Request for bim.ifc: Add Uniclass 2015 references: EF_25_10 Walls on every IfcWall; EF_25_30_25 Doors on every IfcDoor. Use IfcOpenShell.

First a look at what the model holds.

```python
import ifcopenshell

model = ifcopenshell.open("bim.ifc")
print(model.schema)
print("classifications:", [c.Name for c in model.by_type("IfcClassification")])
for ifc_class in ("IfcDoor", "IfcRoof", "IfcStair", "IfcWall", "IfcWindow"):
    print(ifc_class, len(model.by_type(ifc_class)))
```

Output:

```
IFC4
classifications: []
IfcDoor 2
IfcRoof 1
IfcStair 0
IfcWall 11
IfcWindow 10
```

```python
import ifcopenshell
import ifcopenshell.api.classification

model = ifcopenshell.open("bim.ifc")

system = ifcopenshell.api.classification.add_classification(model, classification="Uniclass 2015")

codes = {
    "IfcWall": ("EF_25_10", "Walls"),
    "IfcDoor": ("EF_25_30_25", "Doors"),
}
for ifc_class, (code, name) in codes.items():
    products = model.by_type(ifc_class)
    ifcopenshell.api.classification.add_reference(
        model, products=products, classification=system, identification=code, name=name
    )
    print(code, len(products))

model.write("bim-out.ifc")
```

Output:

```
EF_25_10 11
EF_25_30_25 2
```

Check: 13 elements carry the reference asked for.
